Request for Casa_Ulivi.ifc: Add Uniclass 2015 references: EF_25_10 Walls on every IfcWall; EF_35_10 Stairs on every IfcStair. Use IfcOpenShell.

First a look at what the model holds.

```python
import ifcopenshell

model = ifcopenshell.open("Casa_Ulivi.ifc")
print(model.schema)
print("classifications:", [c.Name for c in model.by_type("IfcClassification")])
for ifc_class in ("IfcDoor", "IfcRoof", "IfcStair", "IfcWall", "IfcWindow"):
    print(ifc_class, len(model.by_type(ifc_class)))
```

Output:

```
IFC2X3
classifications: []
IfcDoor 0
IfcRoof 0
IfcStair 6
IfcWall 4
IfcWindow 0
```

```python
import ifcopenshell
import ifcopenshell.api.classification

model = ifcopenshell.open("Casa_Ulivi.ifc")

# IFC2X3 requires Source and Edition and has no link from the project to the system.
system = model.create_entity("IfcClassification", Source="NBS", Edition="2015", Name="Uniclass 2015")

codes = {
    "IfcWall": ("EF_25_10", "Walls"),
    "IfcStair": ("EF_35_10", "Stairs"),
}
for ifc_class, (code, name) in codes.items():
    products = model.by_type(ifc_class)
    ifcopenshell.api.classification.add_reference(
        model, products=products, classification=system, identification=code, name=name
    )
    print(code, len(products))

model.write("Casa_Ulivi_v2.ifc")
```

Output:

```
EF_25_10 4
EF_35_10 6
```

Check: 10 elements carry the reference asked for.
